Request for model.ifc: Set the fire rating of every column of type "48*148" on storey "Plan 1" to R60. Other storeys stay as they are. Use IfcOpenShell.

First a look at what the model holds.

```python
import ifcopenshell
import ifcopenshell.util.element

model = ifcopenshell.open("model.ifc")
print(model.schema)
storey = next(s for s in model.by_type("IfcBuildingStorey") if s.Name == "Plan 1")
columns = [e for e in ifcopenshell.util.element.get_decomposition(storey) if e.is_a("IfcColumn")]
seen = {}
for e in columns:
    element_type = ifcopenshell.util.element.get_type(e)
    key = (element_type.Name if element_type != e and element_type else None, ifcopenshell.util.element.get_pset(e, "Pset_ColumnCommon", "FireRating"))
    seen[key] = seen.get(key, 0) + 1
for (name, value), count in sorted(seen.items(), key=str):
    print(count, "x", name, "|", value)
```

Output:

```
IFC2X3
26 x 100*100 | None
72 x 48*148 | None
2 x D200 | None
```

```python
import ifcopenshell
import ifcopenshell.api.pset
import ifcopenshell.util.element

model = ifcopenshell.open("model.ifc")

storey = next(s for s in model.by_type("IfcBuildingStorey") if s.Name == "Plan 1")
columns = [e for e in ifcopenshell.util.element.get_decomposition(storey) if e.is_a("IfcColumn")]

count = 0
for e in columns:
    element_type = ifcopenshell.util.element.get_type(e)
    if element_type in (None, e) or element_type.Name != "48*148":
        continue
    found = ifcopenshell.util.element.get_pset(e, "Pset_ColumnCommon", should_inherit=False)
    if found:
        pset = model.by_id(found["id"])
        if len(ifcopenshell.util.element.get_elements_by_pset(pset)) > 1:
            pset = ifcopenshell.api.pset.unshare_pset(model, products=[e], pset=pset)[0]
    else:
        pset = ifcopenshell.api.pset.add_pset(model, product=e, name="Pset_ColumnCommon")
    ifcopenshell.api.pset.edit_pset(model, pset=pset, properties={"FireRating": "R60"})
    count += 1

print(count, "columns updated")

model.write("model_rev.ifc")
```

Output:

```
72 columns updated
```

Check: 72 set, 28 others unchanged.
